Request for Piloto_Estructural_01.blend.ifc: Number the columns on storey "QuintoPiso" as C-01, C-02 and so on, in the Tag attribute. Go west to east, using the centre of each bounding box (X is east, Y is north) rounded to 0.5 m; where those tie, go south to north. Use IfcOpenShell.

First a look at what the model holds.

```python
import ifcopenshell
import ifcopenshell.util.element
import ifcopenshell.util.placement

model = ifcopenshell.open("Piloto_Estructural_01.blend.ifc")
print(model.schema)
storey = next(s for s in model.by_type("IfcBuildingStorey") if s.Name == "QuintoPiso")
columns = [e for e in ifcopenshell.util.element.get_decomposition(storey) if e.is_a("IfcColumn")]
for e in sorted(columns, key=lambda e: e.id()):
    origin = ifcopenshell.util.placement.get_local_placement(e.ObjectPlacement)[:3, 3]
    print(e.id(), e.Tag, e.Name, origin.round(2) + 0.0, sep=" | ")
```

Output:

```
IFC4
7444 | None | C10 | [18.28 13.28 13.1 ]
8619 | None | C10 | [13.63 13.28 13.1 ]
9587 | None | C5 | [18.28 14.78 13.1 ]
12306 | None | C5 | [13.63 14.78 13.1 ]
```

```python
import ifcopenshell
import ifcopenshell.geom
import ifcopenshell.util.element
import ifcopenshell.util.shape

model = ifcopenshell.open("Piloto_Estructural_01.blend.ifc")
settings = ifcopenshell.geom.settings()
settings.set("use-world-coords", True)


def centre(element):
    shape = ifcopenshell.geom.create_shape(settings, element)
    return ifcopenshell.util.shape.get_bbox_centroid(shape.geometry)


storey = next(s for s in model.by_type("IfcBuildingStorey") if s.Name == "QuintoPiso")
columns = [e for e in ifcopenshell.util.element.get_decomposition(storey) if e.is_a("IfcColumn")]

# Insertion points can sit at a corner or the storey origin, so sort by the geometry (in metres).
centres = {e: centre(e) for e in columns}
columns.sort(key=lambda e: (round(centres[e][0] / 0.5), centres[e][1]))

for i, e in enumerate(columns, start=1):
    number = f"C-{i:02d}"
    e.Tag = number
    print(e.id(), number)

model.write("Piloto_Estructural_01.blend_updated.ifc")
```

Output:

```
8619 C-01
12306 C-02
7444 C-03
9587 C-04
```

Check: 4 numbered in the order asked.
